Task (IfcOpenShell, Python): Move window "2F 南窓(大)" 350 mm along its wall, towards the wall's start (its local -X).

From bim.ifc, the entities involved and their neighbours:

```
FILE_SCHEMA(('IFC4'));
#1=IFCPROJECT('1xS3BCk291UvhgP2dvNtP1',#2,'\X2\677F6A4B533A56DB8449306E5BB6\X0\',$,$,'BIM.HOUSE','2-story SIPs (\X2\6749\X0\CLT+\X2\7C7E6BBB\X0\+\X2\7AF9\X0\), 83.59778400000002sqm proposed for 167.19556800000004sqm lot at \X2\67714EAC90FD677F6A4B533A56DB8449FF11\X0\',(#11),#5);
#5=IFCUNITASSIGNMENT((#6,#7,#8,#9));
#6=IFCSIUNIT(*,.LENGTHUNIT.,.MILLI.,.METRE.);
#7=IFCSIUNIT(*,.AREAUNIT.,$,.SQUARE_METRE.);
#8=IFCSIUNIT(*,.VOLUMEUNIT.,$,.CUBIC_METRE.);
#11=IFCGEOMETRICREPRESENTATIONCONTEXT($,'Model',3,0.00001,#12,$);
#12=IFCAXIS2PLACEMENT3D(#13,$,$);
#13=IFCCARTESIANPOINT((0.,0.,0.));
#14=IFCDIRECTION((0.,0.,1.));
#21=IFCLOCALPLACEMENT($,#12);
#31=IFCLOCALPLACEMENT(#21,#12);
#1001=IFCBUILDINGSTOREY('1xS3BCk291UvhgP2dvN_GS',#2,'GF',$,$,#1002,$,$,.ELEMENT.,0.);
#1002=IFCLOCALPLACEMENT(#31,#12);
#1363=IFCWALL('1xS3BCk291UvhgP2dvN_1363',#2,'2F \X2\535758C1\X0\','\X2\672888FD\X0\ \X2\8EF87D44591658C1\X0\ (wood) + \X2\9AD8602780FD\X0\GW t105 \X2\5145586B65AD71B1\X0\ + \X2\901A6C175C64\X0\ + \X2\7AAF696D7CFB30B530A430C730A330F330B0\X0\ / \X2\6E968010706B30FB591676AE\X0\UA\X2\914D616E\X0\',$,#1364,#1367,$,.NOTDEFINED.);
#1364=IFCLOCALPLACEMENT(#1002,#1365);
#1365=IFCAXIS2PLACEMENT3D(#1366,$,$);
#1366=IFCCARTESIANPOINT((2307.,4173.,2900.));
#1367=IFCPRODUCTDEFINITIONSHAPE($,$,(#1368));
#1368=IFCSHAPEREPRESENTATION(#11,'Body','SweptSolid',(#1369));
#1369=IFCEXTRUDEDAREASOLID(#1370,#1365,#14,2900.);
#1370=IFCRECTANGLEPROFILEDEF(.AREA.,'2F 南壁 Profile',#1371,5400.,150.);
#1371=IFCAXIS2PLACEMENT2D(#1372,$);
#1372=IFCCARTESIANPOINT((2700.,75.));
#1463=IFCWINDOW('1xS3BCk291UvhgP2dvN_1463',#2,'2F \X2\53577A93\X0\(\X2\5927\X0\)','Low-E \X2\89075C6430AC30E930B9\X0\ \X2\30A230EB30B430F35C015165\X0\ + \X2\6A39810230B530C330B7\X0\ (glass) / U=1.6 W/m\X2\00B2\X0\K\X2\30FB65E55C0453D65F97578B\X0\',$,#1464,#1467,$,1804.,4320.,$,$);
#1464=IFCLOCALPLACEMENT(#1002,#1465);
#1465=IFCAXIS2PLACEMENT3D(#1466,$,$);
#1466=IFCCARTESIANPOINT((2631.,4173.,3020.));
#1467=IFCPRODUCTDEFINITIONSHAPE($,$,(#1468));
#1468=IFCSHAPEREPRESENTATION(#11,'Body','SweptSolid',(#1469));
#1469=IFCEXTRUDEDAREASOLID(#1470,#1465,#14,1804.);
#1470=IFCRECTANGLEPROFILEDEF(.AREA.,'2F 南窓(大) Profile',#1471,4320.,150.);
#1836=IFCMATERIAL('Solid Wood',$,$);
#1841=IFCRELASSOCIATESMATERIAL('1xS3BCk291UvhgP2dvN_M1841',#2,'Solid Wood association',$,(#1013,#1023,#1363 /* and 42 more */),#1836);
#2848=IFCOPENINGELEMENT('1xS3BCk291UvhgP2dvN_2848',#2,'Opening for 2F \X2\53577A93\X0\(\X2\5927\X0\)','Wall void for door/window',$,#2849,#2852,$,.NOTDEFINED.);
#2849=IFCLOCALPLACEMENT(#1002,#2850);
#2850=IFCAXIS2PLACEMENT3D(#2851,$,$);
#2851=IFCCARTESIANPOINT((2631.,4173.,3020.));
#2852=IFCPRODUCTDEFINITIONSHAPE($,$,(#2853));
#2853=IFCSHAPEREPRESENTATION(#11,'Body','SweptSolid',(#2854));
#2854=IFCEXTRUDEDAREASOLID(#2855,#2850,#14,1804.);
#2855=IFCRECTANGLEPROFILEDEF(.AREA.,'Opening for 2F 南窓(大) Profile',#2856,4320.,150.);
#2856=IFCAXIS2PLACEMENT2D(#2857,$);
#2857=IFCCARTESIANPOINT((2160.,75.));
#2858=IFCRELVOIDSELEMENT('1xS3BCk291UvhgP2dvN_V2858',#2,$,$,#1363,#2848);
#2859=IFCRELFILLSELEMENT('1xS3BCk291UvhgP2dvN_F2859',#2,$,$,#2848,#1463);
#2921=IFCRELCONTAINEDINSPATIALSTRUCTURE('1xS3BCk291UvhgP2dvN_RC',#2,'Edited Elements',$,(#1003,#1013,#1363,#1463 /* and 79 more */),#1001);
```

```python
import ifcopenshell
import ifcopenshell.api.geometry
import ifcopenshell.util.placement

model = ifcopenshell.open("bim.ifc")

window = model.by_guid("1xS3BCk291UvhgP2dvN_1463")
opening = window.FillsVoids[0].RelatingOpeningElement
wall = opening.VoidsElements[0].RelatingBuildingElement

wall_matrix = ifcopenshell.util.placement.get_local_placement(wall.ObjectPlacement)
shift = wall_matrix[:3, 0] * -350.0
before = ifcopenshell.util.placement.get_local_placement(window.ObjectPlacement)[:3, 3].copy()

# The window is not placed relative to its opening, so move both.
for product in (opening, window):
    matrix = ifcopenshell.util.placement.get_local_placement(product.ObjectPlacement)
    matrix[:3, 3] += shift
    ifcopenshell.api.geometry.edit_object_placement(model, product=product, matrix=matrix, is_si=False)

after = ifcopenshell.util.placement.get_local_placement(window.ObjectPlacement)[:3, 3]
print("window moved by", (after - before).round(3) + 0.0)

model.write("bim_rev.ifc")
```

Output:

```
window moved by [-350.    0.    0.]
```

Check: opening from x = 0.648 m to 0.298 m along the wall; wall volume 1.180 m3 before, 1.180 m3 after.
